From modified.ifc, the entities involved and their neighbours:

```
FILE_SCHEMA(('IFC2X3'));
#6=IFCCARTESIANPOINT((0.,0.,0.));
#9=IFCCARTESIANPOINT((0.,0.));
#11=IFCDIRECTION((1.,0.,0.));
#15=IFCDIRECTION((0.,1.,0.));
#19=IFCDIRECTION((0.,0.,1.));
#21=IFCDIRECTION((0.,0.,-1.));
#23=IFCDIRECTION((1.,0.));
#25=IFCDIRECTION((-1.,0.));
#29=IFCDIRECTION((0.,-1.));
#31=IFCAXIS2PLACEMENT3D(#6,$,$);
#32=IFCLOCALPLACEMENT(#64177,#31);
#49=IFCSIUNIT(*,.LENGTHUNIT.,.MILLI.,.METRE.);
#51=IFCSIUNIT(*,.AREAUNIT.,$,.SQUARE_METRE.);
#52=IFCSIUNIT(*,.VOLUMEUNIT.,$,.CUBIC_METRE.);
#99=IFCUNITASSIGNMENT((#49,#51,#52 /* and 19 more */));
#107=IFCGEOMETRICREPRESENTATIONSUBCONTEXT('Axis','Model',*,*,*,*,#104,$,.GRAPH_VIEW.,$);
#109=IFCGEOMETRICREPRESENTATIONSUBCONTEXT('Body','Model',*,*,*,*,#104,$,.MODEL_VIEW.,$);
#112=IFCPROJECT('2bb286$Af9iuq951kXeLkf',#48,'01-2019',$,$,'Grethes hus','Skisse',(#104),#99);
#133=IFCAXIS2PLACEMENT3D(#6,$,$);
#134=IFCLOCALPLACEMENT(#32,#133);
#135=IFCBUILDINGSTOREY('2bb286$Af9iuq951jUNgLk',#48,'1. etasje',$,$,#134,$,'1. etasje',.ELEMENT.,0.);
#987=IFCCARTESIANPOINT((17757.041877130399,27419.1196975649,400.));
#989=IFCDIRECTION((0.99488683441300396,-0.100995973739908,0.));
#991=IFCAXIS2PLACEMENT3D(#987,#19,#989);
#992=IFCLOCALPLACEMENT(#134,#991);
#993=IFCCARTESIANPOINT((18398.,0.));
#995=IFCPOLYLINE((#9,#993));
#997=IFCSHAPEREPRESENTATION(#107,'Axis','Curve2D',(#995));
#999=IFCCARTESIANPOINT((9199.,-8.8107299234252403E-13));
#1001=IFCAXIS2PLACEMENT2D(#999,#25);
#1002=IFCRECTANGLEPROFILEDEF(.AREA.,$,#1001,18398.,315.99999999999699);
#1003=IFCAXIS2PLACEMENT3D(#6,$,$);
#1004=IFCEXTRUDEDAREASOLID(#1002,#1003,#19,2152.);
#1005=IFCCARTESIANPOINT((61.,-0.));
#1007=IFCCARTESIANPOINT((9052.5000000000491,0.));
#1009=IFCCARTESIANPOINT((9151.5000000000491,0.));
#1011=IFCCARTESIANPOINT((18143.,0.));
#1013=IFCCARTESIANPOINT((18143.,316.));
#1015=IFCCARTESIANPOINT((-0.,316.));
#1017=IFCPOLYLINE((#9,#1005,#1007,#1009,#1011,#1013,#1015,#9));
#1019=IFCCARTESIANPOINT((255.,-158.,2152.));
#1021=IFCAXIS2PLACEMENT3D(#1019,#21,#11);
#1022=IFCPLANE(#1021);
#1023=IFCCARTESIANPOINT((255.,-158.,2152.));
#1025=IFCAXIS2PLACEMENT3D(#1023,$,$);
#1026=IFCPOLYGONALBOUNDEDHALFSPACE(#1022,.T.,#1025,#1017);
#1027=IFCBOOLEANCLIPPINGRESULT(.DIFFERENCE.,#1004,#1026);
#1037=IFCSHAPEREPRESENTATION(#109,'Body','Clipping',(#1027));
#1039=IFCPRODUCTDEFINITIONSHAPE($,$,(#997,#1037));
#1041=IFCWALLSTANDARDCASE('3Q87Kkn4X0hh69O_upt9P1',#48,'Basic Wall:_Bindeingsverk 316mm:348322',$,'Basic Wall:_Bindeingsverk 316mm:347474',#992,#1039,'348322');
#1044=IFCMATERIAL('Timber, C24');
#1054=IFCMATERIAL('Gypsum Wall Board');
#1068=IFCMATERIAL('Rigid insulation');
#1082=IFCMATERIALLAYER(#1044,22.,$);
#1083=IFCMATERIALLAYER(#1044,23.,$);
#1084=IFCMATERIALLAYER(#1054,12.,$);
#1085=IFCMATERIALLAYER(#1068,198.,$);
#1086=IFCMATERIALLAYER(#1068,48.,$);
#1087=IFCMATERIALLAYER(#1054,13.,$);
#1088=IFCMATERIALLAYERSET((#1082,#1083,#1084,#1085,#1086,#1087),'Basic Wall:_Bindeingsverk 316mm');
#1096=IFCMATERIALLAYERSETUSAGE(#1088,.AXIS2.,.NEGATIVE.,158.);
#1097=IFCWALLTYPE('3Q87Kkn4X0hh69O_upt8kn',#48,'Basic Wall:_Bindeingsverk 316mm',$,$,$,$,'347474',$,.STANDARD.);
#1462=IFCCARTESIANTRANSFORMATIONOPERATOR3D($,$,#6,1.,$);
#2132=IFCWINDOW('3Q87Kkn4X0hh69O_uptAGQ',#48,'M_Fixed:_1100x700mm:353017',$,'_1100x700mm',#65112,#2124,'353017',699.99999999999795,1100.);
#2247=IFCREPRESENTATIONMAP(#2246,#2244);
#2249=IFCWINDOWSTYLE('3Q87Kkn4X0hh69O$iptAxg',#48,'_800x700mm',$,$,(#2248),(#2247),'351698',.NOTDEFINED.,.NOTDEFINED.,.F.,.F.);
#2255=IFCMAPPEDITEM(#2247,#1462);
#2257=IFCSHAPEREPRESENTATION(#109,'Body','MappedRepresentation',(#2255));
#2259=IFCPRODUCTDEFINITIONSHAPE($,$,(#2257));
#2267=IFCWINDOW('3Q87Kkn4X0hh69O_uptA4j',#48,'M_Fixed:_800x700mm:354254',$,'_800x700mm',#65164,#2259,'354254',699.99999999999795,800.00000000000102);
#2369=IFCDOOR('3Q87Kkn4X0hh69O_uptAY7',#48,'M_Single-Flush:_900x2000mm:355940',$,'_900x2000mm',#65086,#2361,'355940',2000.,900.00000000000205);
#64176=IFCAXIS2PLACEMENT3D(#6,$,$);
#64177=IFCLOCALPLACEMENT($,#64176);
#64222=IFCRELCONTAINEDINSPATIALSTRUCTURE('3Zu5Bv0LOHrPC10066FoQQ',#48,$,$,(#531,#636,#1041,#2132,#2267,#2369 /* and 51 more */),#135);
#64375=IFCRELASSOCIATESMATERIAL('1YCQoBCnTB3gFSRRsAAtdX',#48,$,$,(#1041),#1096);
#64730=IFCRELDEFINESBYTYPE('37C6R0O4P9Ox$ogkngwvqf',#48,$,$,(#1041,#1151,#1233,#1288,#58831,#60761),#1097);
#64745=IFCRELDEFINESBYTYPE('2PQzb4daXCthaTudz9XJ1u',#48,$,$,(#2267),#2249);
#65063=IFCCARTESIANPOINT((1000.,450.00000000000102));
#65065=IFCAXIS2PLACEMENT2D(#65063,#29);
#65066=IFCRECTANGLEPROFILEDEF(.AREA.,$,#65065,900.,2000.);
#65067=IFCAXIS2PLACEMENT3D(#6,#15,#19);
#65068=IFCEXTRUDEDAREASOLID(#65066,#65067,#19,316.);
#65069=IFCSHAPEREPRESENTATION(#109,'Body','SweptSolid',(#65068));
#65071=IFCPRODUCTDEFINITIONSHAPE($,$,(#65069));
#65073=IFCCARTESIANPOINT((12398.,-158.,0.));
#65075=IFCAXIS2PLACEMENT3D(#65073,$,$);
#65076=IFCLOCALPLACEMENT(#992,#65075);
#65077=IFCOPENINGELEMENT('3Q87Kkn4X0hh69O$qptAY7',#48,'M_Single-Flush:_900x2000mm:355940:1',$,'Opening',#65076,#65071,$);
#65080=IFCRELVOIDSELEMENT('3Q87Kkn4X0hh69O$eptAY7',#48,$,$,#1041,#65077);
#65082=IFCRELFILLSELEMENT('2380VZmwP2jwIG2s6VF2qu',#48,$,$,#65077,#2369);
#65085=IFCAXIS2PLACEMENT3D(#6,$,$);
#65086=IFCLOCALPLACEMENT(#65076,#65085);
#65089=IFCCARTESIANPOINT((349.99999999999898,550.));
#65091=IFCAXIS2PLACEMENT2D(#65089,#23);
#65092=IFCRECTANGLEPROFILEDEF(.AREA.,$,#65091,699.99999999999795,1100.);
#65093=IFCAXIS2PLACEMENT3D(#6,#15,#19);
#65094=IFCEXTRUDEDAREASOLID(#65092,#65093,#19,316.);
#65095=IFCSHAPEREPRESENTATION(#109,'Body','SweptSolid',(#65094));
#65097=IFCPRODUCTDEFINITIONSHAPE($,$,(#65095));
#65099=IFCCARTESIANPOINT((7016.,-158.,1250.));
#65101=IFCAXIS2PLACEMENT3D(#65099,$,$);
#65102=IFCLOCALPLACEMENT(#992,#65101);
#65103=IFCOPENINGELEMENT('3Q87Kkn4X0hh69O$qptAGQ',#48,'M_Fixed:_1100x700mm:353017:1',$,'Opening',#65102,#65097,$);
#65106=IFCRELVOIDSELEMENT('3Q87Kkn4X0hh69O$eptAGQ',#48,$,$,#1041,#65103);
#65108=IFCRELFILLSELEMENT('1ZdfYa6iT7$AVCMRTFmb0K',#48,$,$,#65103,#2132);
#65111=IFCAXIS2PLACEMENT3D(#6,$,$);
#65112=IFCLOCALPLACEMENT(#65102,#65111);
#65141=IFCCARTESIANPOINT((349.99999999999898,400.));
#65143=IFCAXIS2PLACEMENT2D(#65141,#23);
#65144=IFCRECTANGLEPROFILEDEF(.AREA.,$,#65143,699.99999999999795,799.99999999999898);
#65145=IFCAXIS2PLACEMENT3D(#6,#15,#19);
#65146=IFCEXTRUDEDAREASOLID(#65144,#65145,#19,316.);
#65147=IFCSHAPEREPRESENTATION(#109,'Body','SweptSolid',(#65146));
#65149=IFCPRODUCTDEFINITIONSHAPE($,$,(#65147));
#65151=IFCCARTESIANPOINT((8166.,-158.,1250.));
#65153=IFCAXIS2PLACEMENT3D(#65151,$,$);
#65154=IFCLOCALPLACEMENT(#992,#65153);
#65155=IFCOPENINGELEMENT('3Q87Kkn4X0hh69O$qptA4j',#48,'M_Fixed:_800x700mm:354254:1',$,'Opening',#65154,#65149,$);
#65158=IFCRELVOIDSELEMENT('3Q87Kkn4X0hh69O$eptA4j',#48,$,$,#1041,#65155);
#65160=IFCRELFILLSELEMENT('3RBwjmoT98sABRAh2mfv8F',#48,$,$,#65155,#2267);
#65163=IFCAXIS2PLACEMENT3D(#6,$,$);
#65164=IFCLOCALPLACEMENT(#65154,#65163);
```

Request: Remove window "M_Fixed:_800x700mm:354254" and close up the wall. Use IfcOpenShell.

```python
import ifcopenshell
import ifcopenshell.api.feature
import ifcopenshell.api.root
import ifcopenshell.geom
import ifcopenshell.util.shape

model = ifcopenshell.open("modified.ifc")
settings = ifcopenshell.geom.settings()


def volume(element):
    """Net volume in cubic metres, openings subtracted."""
    shape = ifcopenshell.geom.create_shape(settings, element)
    return ifcopenshell.util.shape.get_volume(shape.geometry)


window = model.by_guid("3Q87Kkn4X0hh69O_uptA4j")
opening = window.FillsVoids[0].RelatingOpeningElement
wall = opening.VoidsElements[0].RelatingBuildingElement
before = volume(wall)

ifcopenshell.api.root.remove_product(model, product=window)
ifcopenshell.api.feature.remove_feature(model, feature=opening)

after = volume(wall)

print(f"wall volume {before:.3f} -> {after:.3f} m3")

model.write("modified-out.ifc")
```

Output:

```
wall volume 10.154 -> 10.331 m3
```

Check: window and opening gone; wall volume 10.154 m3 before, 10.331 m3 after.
